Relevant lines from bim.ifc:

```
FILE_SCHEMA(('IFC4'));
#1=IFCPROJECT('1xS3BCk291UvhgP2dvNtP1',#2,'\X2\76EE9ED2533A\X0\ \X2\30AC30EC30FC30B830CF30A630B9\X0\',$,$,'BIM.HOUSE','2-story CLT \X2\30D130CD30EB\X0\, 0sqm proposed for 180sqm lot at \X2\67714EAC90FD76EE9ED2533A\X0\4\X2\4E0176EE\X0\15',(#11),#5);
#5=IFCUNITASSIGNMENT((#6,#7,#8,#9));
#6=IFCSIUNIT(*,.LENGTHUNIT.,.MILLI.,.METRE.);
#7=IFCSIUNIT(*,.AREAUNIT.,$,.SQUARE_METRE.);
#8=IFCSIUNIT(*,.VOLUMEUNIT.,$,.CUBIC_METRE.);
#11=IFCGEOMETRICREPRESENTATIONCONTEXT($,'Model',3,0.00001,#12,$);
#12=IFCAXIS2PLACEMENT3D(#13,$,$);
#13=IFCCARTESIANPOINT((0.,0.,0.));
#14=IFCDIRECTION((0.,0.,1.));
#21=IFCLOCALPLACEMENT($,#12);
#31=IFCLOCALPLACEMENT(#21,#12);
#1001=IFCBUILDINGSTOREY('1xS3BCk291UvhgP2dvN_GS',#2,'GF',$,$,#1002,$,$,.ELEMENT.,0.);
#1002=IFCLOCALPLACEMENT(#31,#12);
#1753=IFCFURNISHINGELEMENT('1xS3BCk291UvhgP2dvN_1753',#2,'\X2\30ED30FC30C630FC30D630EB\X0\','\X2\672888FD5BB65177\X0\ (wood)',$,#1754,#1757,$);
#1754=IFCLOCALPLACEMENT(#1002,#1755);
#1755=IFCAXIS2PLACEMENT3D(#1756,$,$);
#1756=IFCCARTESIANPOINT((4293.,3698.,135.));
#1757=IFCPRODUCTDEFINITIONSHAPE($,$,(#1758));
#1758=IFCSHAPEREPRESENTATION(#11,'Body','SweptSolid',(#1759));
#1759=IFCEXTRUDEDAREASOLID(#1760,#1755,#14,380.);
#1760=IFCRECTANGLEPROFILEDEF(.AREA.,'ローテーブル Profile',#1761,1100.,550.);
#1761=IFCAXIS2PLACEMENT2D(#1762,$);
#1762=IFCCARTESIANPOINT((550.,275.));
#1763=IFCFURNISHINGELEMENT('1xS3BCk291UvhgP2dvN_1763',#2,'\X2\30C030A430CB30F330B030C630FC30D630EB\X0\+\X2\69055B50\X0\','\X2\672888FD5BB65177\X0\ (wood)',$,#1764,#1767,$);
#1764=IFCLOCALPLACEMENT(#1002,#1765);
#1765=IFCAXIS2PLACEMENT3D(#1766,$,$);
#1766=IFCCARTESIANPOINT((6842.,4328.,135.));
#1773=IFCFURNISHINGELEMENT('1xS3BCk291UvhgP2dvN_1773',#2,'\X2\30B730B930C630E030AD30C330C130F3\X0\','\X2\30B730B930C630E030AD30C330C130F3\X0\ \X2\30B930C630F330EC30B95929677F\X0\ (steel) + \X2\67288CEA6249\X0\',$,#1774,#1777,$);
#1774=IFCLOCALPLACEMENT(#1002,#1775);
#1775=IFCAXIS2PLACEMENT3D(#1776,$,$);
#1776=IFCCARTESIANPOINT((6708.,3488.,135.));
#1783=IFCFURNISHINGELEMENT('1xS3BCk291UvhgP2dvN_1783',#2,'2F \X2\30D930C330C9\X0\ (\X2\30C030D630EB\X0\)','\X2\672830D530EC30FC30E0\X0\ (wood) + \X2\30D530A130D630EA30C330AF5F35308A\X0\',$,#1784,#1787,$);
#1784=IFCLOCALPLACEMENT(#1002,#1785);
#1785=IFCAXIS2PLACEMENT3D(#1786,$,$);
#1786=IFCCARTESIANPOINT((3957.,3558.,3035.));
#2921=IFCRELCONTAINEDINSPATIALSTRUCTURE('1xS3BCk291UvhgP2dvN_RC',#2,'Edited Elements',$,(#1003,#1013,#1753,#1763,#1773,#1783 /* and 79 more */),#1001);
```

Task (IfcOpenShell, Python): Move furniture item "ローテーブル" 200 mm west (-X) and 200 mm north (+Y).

```python
import ifcopenshell
import ifcopenshell.api.geometry
import ifcopenshell.util.placement
import ifcopenshell.util.unit

model = ifcopenshell.open("bim.ifc")
unit_scale = ifcopenshell.util.unit.calculate_unit_scale(model)

item = model.by_guid("1xS3BCk291UvhgP2dvN_1753")
matrix = ifcopenshell.util.placement.get_local_placement(item.ObjectPlacement)
matrix[0, 3] -= 0.2 / unit_scale
matrix[1, 3] += 0.2 / unit_scale
ifcopenshell.api.geometry.edit_object_placement(model, product=item, matrix=matrix, is_si=False)

print(ifcopenshell.util.placement.get_local_placement(item.ObjectPlacement).round(3) + 0.0)

model.write("bim_rev.ifc")
```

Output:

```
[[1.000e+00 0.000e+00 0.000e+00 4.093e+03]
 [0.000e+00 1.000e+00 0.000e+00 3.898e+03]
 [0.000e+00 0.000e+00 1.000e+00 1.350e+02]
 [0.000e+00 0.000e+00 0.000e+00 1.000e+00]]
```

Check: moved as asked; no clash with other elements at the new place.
